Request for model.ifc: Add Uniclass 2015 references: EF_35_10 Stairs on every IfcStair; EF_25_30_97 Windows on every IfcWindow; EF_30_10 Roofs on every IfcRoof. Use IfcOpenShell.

First a look at what the model holds.

```python
import ifcopenshell

model = ifcopenshell.open("model.ifc")
print(model.schema)
print("classifications:", [c.Name for c in model.by_type("IfcClassification")])
for ifc_class in ("IfcDoor", "IfcRoof", "IfcStair", "IfcWall", "IfcWindow"):
    print(ifc_class, len(model.by_type(ifc_class)))
```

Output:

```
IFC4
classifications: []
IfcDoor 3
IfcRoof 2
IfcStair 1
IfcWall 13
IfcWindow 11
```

```python
import ifcopenshell
import ifcopenshell.api.classification

model = ifcopenshell.open("model.ifc")

system = ifcopenshell.api.classification.add_classification(model, classification="Uniclass 2015")

codes = {
    "IfcStair": ("EF_35_10", "Stairs"),
    "IfcWindow": ("EF_25_30_97", "Windows"),
    "IfcRoof": ("EF_30_10", "Roofs"),
}
for ifc_class, (code, name) in codes.items():
    products = model.by_type(ifc_class)
    ifcopenshell.api.classification.add_reference(
        model, products=products, classification=system, identification=code, name=name
    )
    print(code, len(products))

model.write("model_updated.ifc")
```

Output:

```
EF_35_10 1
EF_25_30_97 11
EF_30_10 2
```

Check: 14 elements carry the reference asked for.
